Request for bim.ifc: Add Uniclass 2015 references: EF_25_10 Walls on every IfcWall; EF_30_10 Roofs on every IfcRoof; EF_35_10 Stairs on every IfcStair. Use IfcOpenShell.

First a look at what the model holds.

```python
import ifcopenshell

model = ifcopenshell.open("bim.ifc")
print(model.schema)
print("classifications:", [c.Name for c in model.by_type("IfcClassification")])
for ifc_class in ("IfcDoor", "IfcRoof", "IfcStair", "IfcWall", "IfcWindow"):
    print(ifc_class, len(model.by_type(ifc_class)))
```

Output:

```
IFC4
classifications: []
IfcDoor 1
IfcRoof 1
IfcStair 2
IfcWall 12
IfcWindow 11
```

```python
import ifcopenshell
import ifcopenshell.api.classification

model = ifcopenshell.open("bim.ifc")

system = ifcopenshell.api.classification.add_classification(model, classification="Uniclass 2015")

codes = {
    "IfcWall": ("EF_25_10", "Walls"),
    "IfcRoof": ("EF_30_10", "Roofs"),
    "IfcStair": ("EF_35_10", "Stairs"),
}
for ifc_class, (code, name) in codes.items():
    products = model.by_type(ifc_class)
    ifcopenshell.api.classification.add_reference(
        model, products=products, classification=system, identification=code, name=name
    )
    print(code, len(products))

model.write("bim_rev.ifc")
```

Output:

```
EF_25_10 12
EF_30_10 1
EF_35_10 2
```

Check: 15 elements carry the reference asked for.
